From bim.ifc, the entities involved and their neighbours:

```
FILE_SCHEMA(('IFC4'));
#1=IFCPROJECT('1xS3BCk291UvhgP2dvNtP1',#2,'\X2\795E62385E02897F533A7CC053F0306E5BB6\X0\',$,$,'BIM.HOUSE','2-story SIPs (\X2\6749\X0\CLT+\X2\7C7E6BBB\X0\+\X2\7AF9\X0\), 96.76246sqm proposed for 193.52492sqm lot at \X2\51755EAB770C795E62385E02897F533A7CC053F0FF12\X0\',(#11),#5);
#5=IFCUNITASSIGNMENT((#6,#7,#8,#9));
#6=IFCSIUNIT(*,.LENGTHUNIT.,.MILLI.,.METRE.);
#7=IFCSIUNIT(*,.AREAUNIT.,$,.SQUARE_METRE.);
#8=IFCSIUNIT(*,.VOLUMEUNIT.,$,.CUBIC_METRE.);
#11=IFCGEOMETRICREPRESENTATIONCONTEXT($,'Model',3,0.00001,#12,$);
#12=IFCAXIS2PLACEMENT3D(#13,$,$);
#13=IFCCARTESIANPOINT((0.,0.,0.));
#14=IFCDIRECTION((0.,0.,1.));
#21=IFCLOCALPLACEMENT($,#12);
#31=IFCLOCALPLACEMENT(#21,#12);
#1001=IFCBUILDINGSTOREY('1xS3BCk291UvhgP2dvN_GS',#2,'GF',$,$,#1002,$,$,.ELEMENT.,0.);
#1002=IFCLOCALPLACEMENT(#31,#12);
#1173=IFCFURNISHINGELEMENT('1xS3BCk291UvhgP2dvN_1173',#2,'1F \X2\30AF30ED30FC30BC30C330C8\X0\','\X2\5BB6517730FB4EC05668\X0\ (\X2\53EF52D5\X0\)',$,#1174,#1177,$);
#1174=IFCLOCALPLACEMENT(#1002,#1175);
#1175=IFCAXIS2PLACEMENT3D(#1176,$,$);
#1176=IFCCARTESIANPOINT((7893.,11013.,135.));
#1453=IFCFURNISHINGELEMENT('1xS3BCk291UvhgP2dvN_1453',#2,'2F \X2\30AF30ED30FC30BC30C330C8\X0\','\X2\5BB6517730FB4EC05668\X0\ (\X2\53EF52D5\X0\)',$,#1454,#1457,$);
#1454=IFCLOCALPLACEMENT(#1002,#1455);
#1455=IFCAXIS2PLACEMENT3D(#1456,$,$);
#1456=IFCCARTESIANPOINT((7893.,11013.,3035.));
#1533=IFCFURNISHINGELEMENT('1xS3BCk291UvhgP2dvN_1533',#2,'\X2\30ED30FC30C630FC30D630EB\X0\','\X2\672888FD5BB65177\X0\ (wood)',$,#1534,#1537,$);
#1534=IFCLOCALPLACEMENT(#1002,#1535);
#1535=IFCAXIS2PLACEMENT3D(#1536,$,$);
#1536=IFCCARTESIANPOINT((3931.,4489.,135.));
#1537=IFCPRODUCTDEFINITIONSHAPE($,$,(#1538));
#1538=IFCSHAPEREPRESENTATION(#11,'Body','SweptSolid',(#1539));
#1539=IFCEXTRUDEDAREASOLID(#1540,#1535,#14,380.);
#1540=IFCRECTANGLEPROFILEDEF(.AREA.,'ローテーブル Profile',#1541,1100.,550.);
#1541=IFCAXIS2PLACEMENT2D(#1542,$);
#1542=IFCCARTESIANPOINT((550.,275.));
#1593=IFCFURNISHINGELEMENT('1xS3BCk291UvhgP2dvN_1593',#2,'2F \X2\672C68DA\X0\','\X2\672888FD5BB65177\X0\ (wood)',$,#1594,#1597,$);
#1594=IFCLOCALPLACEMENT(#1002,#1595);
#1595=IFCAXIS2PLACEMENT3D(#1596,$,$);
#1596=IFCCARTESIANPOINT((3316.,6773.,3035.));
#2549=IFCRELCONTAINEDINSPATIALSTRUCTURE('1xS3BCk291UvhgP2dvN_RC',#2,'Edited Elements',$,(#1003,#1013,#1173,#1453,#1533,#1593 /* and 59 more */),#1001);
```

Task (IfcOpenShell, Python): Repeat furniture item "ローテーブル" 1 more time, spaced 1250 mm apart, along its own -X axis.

```python
import ifcopenshell
import ifcopenshell.api.geometry
import ifcopenshell.api.root
import ifcopenshell.util.element
import ifcopenshell.util.placement
import ifcopenshell.util.unit

model = ifcopenshell.open("bim.ifc")
unit_scale = ifcopenshell.util.unit.calculate_unit_scale(model)


def reuse_history(source, copy):
    """copy_class also copies each property set's owner history, people and application; keep the originals."""
    for rel in copy.IsDefinedBy:
        if rel.is_a("IfcRelDefinesByProperties") and (history := rel.RelatingPropertyDefinition.OwnerHistory):
            rel.RelatingPropertyDefinition.OwnerHistory = source.OwnerHistory
            ifcopenshell.util.element.remove_deep2(model, history)


source = model.by_id(1533)
base = ifcopenshell.util.placement.get_local_placement(source.ObjectPlacement)
step = -base[:3, 0] * 1.25 / unit_scale

for i in range(1, 2):
    copy = ifcopenshell.api.root.copy_class(model, product=source)
    copy.Representation = ifcopenshell.util.element.copy_deep(
        model, source.Representation, exclude=["IfcGeometricRepresentationContext", "IfcRepresentationMap"]
    )
    reuse_history(source, copy)
    matrix = base.copy()
    matrix[:3, 3] += i * step
    print("added at", matrix[:3, 3].round(3) + 0.0)
    ifcopenshell.api.geometry.edit_object_placement(model, product=copy, matrix=matrix, is_si=False)

model.write("bim_updated.ifc")
```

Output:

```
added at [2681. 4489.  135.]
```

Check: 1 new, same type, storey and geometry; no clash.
